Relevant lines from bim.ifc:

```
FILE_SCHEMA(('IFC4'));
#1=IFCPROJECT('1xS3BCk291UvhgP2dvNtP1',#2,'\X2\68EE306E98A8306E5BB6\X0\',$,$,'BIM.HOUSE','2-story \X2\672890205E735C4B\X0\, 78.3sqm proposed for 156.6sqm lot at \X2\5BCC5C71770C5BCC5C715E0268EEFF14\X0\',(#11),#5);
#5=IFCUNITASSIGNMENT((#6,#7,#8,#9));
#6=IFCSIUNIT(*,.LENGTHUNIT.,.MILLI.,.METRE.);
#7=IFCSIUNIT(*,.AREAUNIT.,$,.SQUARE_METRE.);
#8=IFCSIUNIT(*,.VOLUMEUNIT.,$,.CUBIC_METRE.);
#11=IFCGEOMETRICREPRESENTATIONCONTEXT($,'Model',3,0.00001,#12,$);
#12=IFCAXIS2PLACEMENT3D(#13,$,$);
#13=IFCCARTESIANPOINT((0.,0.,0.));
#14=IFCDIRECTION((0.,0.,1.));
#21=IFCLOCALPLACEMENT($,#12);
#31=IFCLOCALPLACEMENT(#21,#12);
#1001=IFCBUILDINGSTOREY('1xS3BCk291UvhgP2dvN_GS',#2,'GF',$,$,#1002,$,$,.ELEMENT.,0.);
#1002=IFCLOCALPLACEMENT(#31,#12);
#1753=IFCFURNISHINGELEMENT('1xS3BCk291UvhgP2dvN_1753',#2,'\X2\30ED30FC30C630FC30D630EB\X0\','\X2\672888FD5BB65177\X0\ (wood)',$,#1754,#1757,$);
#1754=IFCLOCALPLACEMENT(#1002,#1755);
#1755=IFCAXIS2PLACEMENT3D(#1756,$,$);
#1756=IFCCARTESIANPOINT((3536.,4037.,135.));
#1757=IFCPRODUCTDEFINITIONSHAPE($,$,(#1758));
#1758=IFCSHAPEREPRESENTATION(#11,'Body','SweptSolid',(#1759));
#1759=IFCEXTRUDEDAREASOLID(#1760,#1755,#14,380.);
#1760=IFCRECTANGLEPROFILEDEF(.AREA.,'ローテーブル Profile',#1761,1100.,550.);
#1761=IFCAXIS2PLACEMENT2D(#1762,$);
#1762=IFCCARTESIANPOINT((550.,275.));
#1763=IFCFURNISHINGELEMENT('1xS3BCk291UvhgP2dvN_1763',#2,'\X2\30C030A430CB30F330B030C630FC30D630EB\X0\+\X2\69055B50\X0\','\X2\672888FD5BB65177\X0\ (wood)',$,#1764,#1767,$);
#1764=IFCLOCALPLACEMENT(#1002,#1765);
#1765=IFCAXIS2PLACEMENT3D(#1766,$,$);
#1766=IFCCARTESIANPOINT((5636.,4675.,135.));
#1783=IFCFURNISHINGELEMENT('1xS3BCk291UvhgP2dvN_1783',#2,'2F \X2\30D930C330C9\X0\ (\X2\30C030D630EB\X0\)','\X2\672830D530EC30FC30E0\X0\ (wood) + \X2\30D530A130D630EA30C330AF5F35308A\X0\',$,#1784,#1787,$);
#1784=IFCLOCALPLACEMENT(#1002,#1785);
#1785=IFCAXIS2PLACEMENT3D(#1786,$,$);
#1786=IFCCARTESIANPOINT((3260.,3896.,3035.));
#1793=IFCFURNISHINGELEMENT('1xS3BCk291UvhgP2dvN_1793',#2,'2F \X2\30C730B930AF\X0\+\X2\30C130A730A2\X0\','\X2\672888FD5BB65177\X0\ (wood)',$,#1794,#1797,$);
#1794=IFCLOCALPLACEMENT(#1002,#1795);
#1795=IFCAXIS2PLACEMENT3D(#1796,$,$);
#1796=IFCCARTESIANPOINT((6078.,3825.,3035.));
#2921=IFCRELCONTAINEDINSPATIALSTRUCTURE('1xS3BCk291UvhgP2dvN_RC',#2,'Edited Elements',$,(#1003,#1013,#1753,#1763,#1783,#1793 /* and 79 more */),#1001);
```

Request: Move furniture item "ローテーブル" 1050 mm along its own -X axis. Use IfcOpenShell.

```python
import ifcopenshell
import ifcopenshell.api.geometry
import ifcopenshell.util.placement
import ifcopenshell.util.unit

model = ifcopenshell.open("bim.ifc")
unit_scale = ifcopenshell.util.unit.calculate_unit_scale(model)

item = model.by_guid("1xS3BCk291UvhgP2dvN_1753")
matrix = ifcopenshell.util.placement.get_local_placement(item.ObjectPlacement)
matrix[:3, 3] -= matrix[:3, 0] * 1.05 / unit_scale
ifcopenshell.api.geometry.edit_object_placement(model, product=item, matrix=matrix, is_si=False)

print(ifcopenshell.util.placement.get_local_placement(item.ObjectPlacement).round(3) + 0.0)

model.write("bim_edited.ifc")
```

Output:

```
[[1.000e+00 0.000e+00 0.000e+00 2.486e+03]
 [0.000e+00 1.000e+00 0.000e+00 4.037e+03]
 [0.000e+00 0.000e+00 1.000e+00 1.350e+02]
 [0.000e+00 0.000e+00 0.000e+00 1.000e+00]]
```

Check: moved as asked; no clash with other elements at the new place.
